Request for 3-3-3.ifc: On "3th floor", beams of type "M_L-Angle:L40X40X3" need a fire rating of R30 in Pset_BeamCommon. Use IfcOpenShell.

First a look at what the model holds.

```python
import ifcopenshell
import ifcopenshell.util.element

model = ifcopenshell.open("3-3-3.ifc")
print(model.schema)
storey = next(s for s in model.by_type("IfcBuildingStorey") if s.Name == "3th floor")
beams = [e for e in ifcopenshell.util.element.get_decomposition(storey) if e.is_a("IfcBeam")]
seen = {}
for e in beams:
    element_type = ifcopenshell.util.element.get_type(e)
    key = (element_type.Name if element_type != e and element_type else None, ifcopenshell.util.element.get_pset(e, "Pset_BeamCommon", "FireRating"))
    seen[key] = seen.get(key, 0) + 1
for (name, value), count in sorted(seen.items(), key=str):
    print(count, "x", name, "|", value)
```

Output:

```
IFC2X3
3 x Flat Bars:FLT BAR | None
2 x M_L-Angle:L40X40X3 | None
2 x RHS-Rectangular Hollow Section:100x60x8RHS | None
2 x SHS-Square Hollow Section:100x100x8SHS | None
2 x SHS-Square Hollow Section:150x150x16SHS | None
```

```python
import ifcopenshell
import ifcopenshell.api.pset
import ifcopenshell.util.element

model = ifcopenshell.open("3-3-3.ifc")

storey = next(s for s in model.by_type("IfcBuildingStorey") if s.Name == "3th floor")
beams = [e for e in ifcopenshell.util.element.get_decomposition(storey) if e.is_a("IfcBeam")]

count = 0
for e in beams:
    element_type = ifcopenshell.util.element.get_type(e)
    if element_type in (None, e) or element_type.Name != "M_L-Angle:L40X40X3":
        continue
    # add_pset returns the element's existing set when there is one.
    pset = ifcopenshell.api.pset.add_pset(model, product=e, name="Pset_BeamCommon")
    ifcopenshell.api.pset.edit_pset(model, pset=pset, properties={"FireRating": "R30"})
    count += 1

print(count, "beams updated")

model.write("3-3-3_updated.ifc")
```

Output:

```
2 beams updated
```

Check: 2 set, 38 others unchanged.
